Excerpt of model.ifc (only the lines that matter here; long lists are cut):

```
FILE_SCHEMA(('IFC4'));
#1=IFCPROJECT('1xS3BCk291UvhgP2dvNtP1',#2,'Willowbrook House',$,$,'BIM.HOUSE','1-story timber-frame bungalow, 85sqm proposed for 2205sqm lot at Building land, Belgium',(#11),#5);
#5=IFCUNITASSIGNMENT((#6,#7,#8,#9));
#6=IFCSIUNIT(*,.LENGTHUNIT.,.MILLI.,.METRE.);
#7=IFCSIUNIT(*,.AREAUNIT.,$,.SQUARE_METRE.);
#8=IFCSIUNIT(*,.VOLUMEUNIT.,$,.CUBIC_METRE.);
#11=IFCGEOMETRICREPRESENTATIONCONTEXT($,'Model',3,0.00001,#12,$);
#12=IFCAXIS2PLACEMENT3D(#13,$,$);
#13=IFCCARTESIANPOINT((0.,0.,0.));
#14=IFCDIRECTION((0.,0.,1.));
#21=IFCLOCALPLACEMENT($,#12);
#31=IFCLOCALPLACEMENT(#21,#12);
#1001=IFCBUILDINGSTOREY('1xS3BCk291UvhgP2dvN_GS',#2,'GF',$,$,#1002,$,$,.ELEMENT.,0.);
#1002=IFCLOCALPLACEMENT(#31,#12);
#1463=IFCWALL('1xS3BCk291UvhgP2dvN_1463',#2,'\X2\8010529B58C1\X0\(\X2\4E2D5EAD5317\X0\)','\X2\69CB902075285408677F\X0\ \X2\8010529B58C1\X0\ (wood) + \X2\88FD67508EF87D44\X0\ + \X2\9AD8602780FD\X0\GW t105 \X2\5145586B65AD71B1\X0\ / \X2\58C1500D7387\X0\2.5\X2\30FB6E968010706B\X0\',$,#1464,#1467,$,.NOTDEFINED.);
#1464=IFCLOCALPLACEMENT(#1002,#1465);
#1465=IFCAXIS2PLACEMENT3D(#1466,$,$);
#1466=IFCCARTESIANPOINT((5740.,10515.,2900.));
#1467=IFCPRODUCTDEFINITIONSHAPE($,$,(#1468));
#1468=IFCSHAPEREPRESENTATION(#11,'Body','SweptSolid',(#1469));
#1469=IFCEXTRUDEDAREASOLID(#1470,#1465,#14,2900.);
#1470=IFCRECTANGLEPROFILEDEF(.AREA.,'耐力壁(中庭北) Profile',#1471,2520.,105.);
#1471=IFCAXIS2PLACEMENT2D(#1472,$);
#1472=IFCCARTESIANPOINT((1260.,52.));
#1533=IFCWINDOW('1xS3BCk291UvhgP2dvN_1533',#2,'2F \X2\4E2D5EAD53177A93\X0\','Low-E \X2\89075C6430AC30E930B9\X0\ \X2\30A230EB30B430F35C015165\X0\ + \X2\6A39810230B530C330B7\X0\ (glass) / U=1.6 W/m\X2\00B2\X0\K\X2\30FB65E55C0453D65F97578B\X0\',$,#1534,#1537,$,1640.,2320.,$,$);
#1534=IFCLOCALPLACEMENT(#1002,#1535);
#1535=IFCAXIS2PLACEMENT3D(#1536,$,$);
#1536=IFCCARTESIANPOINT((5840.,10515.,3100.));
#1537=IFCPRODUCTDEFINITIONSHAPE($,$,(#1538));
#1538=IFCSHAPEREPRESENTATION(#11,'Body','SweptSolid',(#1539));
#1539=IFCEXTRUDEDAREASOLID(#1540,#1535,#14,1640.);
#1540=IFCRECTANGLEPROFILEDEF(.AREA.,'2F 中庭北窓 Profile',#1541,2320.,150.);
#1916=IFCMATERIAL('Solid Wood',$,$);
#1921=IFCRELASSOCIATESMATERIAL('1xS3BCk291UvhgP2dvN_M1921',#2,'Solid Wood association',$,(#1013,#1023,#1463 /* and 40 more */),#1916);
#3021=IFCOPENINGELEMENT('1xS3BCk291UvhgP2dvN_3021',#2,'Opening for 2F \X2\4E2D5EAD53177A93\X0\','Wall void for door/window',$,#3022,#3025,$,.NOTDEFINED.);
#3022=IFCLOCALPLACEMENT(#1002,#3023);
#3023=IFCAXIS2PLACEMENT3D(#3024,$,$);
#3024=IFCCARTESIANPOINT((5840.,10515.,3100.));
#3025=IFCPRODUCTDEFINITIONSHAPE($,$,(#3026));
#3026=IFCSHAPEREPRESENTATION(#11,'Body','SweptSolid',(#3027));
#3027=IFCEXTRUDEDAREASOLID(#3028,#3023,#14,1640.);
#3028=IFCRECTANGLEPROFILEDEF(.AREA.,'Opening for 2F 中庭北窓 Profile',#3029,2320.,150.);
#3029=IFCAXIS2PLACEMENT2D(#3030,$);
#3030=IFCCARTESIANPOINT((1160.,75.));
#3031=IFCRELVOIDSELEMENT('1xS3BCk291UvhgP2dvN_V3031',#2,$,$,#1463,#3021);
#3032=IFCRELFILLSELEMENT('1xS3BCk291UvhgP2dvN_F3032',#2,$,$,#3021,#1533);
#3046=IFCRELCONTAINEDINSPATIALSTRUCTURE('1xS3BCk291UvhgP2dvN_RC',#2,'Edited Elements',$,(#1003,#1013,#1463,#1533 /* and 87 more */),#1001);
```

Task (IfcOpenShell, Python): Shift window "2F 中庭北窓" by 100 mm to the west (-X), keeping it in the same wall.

```python
import ifcopenshell
import ifcopenshell.api.geometry
import ifcopenshell.util.placement
import ifcopenshell.util.unit

model = ifcopenshell.open("model.ifc")
unit_scale = ifcopenshell.util.unit.calculate_unit_scale(model)

window = model.by_id(1533)
opening = window.FillsVoids[0].RelatingOpeningElement
wall = opening.VoidsElements[0].RelatingBuildingElement

wall_matrix = ifcopenshell.util.placement.get_local_placement(wall.ObjectPlacement)
shift = wall_matrix[:3, 0] * -0.1 / unit_scale
before = ifcopenshell.util.placement.get_local_placement(window.ObjectPlacement)[:3, 3].copy()

# The window is not placed relative to its opening, so move both.
for product in (opening, window):
    matrix = ifcopenshell.util.placement.get_local_placement(product.ObjectPlacement)
    matrix[:3, 3] += shift
    ifcopenshell.api.geometry.edit_object_placement(model, product=product, matrix=matrix, is_si=False)

after = ifcopenshell.util.placement.get_local_placement(window.ObjectPlacement)[:3, 3]
print("window moved by", (after - before).round(3) + 0.0)

model.write("model_v2.ifc")
```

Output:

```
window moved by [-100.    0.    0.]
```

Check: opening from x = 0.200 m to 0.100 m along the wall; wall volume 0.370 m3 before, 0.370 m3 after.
